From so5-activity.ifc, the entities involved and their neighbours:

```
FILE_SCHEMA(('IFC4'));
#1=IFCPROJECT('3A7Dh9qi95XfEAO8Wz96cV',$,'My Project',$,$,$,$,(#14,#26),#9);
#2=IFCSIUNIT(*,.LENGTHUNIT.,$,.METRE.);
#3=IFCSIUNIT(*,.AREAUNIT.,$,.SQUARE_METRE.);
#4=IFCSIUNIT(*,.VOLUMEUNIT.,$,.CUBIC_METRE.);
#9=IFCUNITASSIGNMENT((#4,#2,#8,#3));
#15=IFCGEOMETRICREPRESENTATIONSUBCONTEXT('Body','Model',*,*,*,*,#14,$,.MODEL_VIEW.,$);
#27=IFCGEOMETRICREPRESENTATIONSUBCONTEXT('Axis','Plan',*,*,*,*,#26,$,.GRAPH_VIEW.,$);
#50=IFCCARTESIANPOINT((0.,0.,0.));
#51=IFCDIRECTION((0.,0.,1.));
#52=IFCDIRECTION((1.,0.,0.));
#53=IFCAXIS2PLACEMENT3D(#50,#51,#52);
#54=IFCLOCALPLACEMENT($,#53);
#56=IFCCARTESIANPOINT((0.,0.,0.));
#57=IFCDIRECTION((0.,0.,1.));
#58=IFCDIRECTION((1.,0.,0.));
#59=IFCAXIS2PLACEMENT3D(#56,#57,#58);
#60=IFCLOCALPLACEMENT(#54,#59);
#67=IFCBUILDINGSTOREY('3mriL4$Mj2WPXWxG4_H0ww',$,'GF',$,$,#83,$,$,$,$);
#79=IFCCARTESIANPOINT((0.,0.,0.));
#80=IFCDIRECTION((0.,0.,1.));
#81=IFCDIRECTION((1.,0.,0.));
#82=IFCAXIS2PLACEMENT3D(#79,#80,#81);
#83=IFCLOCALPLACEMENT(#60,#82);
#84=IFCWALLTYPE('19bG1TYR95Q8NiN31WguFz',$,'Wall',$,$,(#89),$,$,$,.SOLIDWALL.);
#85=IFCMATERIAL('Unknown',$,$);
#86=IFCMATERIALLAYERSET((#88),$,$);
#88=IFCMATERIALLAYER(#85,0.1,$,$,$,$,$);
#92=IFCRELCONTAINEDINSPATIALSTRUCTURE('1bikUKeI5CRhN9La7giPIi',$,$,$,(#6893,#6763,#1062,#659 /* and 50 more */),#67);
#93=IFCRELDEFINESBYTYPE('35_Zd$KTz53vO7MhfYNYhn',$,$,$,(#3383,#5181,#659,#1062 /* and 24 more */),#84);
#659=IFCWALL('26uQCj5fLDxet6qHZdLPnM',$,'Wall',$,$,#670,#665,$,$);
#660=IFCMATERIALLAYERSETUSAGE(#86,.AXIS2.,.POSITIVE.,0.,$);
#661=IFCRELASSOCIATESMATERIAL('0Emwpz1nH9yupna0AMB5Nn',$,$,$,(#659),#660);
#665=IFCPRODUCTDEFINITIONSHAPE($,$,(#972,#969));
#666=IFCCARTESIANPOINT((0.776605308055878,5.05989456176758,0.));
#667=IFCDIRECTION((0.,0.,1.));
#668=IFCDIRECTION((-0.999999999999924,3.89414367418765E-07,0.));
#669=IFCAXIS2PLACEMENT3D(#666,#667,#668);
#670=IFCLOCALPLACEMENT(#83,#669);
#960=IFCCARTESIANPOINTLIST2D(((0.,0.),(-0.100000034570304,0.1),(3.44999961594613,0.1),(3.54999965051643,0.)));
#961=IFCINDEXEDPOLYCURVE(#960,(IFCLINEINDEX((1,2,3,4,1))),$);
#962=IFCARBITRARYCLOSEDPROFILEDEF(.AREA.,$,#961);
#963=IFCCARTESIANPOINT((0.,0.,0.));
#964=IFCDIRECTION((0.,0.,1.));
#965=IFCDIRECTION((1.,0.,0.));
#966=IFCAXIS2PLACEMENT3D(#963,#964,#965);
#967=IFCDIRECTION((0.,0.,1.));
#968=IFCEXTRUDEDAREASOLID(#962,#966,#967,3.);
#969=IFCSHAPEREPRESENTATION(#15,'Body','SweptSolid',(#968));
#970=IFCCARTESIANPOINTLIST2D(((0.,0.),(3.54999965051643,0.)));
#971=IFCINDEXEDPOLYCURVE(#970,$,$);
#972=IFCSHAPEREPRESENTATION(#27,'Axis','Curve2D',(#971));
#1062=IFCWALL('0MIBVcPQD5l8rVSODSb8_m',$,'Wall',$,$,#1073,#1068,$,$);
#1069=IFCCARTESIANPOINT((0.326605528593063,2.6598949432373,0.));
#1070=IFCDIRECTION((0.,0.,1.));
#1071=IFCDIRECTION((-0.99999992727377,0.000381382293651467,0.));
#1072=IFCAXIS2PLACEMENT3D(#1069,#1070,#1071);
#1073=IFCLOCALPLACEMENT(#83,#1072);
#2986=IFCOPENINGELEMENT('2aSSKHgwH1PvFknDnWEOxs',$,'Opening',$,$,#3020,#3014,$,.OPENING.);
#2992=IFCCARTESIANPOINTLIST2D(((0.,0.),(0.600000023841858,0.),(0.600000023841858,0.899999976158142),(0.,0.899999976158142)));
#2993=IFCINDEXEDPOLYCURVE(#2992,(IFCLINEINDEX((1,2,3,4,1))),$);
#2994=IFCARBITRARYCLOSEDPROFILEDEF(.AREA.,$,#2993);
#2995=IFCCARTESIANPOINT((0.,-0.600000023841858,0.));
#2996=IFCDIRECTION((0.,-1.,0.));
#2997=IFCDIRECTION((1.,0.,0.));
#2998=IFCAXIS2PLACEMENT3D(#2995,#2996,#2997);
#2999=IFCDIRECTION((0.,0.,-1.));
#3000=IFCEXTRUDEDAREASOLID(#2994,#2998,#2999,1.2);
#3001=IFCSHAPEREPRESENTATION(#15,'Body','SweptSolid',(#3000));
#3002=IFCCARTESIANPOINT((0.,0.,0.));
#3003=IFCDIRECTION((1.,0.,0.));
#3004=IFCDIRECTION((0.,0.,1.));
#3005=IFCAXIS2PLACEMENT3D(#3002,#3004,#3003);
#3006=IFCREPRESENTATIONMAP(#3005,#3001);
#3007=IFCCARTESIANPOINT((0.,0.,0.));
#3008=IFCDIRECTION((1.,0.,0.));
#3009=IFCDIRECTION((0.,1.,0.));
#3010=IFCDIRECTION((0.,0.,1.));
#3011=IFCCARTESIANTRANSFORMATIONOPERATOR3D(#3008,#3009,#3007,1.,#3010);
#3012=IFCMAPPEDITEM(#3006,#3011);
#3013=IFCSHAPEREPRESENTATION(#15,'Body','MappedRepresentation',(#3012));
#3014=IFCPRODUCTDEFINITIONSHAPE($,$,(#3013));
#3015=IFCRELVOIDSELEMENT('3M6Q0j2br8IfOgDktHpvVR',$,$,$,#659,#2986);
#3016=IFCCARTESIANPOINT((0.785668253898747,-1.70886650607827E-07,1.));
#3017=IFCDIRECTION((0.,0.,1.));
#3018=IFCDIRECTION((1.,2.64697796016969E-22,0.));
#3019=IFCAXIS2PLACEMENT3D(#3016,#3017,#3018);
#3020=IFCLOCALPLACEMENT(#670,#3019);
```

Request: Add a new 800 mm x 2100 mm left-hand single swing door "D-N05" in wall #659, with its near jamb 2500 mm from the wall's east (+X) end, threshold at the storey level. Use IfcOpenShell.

```python
import numpy as np
import ifcopenshell
import ifcopenshell.api.feature
import ifcopenshell.api.geometry
import ifcopenshell.api.root
import ifcopenshell.api.spatial
import ifcopenshell.geom
import ifcopenshell.util.element
import ifcopenshell.util.placement
import ifcopenshell.util.representation
import ifcopenshell.util.shape
import ifcopenshell.util.unit

model = ifcopenshell.open("so5-activity.ifc")
unit_scale = ifcopenshell.util.unit.calculate_unit_scale(model)
settings = ifcopenshell.geom.settings()


def volume(element):
    """Net volume in cubic metres, openings subtracted."""
    shape = ifcopenshell.geom.create_shape(settings, element)
    return ifcopenshell.util.shape.get_volume(shape.geometry)


wall = model.by_id(659)
storey = ifcopenshell.util.element.get_container(wall, ifc_class="IfcBuildingStorey")
context = ifcopenshell.util.representation.get_context(model, "Model", "Body", "MODEL_VIEW")
before = volume(wall)

width, height, from_end, sill = 0.8, 2.1, 2.5, 0.0  # metres

# The wall runs along its own X axis, and the end named is its -X end.
wall_shape = ifcopenshell.geom.create_shape(settings, wall)
x, y, z = ifcopenshell.util.shape.get_vertices(wall_shape.geometry).T
start = x.min() + from_end
face, thickness = float(y.min()), float(y.max() - y.min())
wall_matrix = ifcopenshell.util.placement.get_local_placement(wall.ObjectPlacement)
level = ifcopenshell.util.placement.get_local_placement(storey.ObjectPlacement)[2, 3]


def in_wall(x, y):
    """Placement at x, y metres in the wall's axes, at sill height."""
    matrix = wall_matrix.copy()
    matrix[:, 3] = wall_matrix @ np.array([x / unit_scale, y / unit_scale, 0.0, 1.0])
    matrix[2, 3] = level + sill / unit_scale
    return matrix


# Opening: a box that overshoots both wall faces by 50 mm.
opening = ifcopenshell.api.root.create_entity(model, ifc_class="IfcOpeningElement", predefined_type="OPENING")
box = ifcopenshell.api.geometry.add_wall_representation(
    model, context=context, length=width, height=height, thickness=thickness + 0.1
)
ifcopenshell.api.geometry.assign_representation(model, product=opening, representation=box)
ifcopenshell.api.geometry.edit_object_placement(model, product=opening, matrix=in_wall(start, face - 0.05), is_si=False)
ifcopenshell.api.feature.add_feature(model, feature=opening, element=wall)

door = ifcopenshell.api.root.create_entity(model, ifc_class="IfcDoor", name="D-N05", predefined_type="DOOR")
door.OverallWidth, door.OverallHeight = width / unit_scale, height / unit_scale
door.OperationType = "SINGLE_SWING_LEFT"
body = ifcopenshell.api.geometry.add_door_representation(
    model,
    context=context,
    overall_width=door.OverallWidth,
    overall_height=door.OverallHeight,
    operation_type="SINGLE_SWING_LEFT",
    lining_properties={"LiningDepth": thickness / unit_scale, "ThresholdDepth": thickness / unit_scale},
)
ifcopenshell.api.geometry.assign_representation(model, product=door, representation=body)
ifcopenshell.api.spatial.assign_container(model, products=[door], relating_structure=storey)
ifcopenshell.api.feature.add_filling(model, opening=opening, element=door)

# The lining spans the wall, so the door starts at the wall face.
ifcopenshell.api.geometry.edit_object_placement(model, product=door, matrix=in_wall(start, face), is_si=False)

after = volume(wall)

print(f"wall volume {before:.3f} -> {after:.3f} m3")

model.write("so5-activity-out.ifc")
```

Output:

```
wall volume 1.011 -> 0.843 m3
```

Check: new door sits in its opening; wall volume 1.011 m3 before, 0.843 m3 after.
